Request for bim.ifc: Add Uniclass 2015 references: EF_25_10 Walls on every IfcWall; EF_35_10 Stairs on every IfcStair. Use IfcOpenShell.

First a look at what the model holds.

```python
import ifcopenshell

model = ifcopenshell.open("bim.ifc")
print(model.schema)
print("classifications:", [c.Name for c in model.by_type("IfcClassification")])
for ifc_class in ("IfcDoor", "IfcRoof", "IfcStair", "IfcWall", "IfcWindow"):
    print(ifc_class, len(model.by_type(ifc_class)))
```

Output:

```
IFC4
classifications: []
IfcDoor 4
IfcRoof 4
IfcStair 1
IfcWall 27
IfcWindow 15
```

```python
import ifcopenshell
import ifcopenshell.api.classification

model = ifcopenshell.open("bim.ifc")

system = ifcopenshell.api.classification.add_classification(model, classification="Uniclass 2015")

codes = {
    "IfcWall": ("EF_25_10", "Walls"),
    "IfcStair": ("EF_35_10", "Stairs"),
}
for ifc_class, (code, name) in codes.items():
    products = model.by_type(ifc_class)
    ifcopenshell.api.classification.add_reference(
        model, products=products, classification=system, identification=code, name=name
    )
    print(code, len(products))

model.write("bim_rev.ifc")
```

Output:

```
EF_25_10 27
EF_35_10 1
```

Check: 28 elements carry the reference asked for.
